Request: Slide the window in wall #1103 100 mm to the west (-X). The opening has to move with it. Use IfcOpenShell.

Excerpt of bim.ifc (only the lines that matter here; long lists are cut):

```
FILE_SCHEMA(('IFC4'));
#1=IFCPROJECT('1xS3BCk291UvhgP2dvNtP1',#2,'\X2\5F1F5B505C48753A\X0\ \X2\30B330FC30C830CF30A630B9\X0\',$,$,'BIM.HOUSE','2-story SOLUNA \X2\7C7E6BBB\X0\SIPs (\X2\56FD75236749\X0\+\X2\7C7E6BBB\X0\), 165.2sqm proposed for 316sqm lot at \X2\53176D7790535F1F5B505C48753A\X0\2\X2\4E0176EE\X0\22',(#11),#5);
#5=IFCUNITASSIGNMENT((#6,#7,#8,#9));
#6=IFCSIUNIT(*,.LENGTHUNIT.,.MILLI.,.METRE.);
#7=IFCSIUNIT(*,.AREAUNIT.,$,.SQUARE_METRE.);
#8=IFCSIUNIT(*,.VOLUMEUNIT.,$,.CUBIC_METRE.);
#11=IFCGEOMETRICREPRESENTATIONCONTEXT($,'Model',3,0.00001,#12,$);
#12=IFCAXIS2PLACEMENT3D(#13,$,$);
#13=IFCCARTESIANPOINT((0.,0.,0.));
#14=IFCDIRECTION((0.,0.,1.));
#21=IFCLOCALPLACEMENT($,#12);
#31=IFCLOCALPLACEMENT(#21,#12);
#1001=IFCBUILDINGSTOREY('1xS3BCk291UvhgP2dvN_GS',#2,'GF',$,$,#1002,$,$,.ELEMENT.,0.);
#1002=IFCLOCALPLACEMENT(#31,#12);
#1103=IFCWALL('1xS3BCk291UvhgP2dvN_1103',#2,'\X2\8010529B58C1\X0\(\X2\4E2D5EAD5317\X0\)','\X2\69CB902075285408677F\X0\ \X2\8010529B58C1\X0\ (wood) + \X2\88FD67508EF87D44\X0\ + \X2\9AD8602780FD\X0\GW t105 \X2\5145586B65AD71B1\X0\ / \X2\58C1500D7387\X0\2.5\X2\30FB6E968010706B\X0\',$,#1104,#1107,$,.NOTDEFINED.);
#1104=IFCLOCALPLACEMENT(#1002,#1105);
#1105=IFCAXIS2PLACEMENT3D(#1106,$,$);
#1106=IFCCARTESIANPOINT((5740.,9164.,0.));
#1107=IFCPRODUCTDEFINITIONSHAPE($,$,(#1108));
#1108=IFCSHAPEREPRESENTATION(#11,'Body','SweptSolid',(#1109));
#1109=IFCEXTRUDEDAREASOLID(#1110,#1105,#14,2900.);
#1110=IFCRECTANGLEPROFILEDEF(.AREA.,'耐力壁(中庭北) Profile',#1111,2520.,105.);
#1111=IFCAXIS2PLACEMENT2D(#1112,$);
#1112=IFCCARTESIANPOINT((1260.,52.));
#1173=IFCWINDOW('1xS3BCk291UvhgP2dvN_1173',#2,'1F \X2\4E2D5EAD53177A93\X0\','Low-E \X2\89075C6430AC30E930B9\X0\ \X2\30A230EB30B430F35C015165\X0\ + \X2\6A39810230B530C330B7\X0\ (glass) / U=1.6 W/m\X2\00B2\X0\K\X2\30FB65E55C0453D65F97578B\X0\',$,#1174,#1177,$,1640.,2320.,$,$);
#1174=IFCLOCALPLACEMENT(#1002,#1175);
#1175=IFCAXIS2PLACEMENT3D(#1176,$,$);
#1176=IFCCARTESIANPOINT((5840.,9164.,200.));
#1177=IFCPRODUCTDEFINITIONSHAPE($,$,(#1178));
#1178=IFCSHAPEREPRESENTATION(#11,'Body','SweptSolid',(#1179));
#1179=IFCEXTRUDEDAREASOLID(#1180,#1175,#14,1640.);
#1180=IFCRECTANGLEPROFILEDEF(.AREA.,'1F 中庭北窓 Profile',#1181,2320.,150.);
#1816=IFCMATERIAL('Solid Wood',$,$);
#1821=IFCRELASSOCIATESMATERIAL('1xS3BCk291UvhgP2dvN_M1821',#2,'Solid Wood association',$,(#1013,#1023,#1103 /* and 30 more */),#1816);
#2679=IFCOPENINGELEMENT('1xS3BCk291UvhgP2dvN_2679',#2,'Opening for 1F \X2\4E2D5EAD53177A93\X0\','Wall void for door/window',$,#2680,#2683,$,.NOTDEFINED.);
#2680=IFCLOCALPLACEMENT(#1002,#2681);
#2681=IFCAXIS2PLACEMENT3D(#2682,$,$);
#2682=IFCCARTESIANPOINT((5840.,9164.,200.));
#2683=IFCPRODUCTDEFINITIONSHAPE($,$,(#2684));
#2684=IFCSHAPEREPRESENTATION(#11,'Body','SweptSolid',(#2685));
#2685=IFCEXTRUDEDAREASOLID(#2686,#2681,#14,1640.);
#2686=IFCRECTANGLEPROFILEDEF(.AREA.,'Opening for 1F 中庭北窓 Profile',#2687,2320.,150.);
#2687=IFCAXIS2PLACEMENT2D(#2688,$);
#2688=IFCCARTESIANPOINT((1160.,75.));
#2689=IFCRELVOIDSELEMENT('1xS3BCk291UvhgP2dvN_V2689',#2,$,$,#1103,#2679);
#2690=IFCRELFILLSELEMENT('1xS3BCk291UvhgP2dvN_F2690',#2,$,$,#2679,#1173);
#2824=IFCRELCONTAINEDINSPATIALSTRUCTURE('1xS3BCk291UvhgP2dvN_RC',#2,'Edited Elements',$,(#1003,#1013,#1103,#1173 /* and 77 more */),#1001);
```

```python
import ifcopenshell
import ifcopenshell.api.geometry
import ifcopenshell.util.placement

model = ifcopenshell.open("bim.ifc")

window = model.by_guid("1xS3BCk291UvhgP2dvN_1173")
opening = window.FillsVoids[0].RelatingOpeningElement
wall = opening.VoidsElements[0].RelatingBuildingElement

wall_matrix = ifcopenshell.util.placement.get_local_placement(wall.ObjectPlacement)
shift = wall_matrix[:3, 0] * -100.0
before = ifcopenshell.util.placement.get_local_placement(window.ObjectPlacement)[:3, 3].copy()

# The window is not placed relative to its opening, so move both.
for product in (opening, window):
    matrix = ifcopenshell.util.placement.get_local_placement(product.ObjectPlacement)
    matrix[:3, 3] += shift
    ifcopenshell.api.geometry.edit_object_placement(model, product=product, matrix=matrix, is_si=False)

after = ifcopenshell.util.placement.get_local_placement(window.ObjectPlacement)[:3, 3]
print("window moved by", (after - before).round(3) + 0.0)

model.write("bim-out.ifc")
```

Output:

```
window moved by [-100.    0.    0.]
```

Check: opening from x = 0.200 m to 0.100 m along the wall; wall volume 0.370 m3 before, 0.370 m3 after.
